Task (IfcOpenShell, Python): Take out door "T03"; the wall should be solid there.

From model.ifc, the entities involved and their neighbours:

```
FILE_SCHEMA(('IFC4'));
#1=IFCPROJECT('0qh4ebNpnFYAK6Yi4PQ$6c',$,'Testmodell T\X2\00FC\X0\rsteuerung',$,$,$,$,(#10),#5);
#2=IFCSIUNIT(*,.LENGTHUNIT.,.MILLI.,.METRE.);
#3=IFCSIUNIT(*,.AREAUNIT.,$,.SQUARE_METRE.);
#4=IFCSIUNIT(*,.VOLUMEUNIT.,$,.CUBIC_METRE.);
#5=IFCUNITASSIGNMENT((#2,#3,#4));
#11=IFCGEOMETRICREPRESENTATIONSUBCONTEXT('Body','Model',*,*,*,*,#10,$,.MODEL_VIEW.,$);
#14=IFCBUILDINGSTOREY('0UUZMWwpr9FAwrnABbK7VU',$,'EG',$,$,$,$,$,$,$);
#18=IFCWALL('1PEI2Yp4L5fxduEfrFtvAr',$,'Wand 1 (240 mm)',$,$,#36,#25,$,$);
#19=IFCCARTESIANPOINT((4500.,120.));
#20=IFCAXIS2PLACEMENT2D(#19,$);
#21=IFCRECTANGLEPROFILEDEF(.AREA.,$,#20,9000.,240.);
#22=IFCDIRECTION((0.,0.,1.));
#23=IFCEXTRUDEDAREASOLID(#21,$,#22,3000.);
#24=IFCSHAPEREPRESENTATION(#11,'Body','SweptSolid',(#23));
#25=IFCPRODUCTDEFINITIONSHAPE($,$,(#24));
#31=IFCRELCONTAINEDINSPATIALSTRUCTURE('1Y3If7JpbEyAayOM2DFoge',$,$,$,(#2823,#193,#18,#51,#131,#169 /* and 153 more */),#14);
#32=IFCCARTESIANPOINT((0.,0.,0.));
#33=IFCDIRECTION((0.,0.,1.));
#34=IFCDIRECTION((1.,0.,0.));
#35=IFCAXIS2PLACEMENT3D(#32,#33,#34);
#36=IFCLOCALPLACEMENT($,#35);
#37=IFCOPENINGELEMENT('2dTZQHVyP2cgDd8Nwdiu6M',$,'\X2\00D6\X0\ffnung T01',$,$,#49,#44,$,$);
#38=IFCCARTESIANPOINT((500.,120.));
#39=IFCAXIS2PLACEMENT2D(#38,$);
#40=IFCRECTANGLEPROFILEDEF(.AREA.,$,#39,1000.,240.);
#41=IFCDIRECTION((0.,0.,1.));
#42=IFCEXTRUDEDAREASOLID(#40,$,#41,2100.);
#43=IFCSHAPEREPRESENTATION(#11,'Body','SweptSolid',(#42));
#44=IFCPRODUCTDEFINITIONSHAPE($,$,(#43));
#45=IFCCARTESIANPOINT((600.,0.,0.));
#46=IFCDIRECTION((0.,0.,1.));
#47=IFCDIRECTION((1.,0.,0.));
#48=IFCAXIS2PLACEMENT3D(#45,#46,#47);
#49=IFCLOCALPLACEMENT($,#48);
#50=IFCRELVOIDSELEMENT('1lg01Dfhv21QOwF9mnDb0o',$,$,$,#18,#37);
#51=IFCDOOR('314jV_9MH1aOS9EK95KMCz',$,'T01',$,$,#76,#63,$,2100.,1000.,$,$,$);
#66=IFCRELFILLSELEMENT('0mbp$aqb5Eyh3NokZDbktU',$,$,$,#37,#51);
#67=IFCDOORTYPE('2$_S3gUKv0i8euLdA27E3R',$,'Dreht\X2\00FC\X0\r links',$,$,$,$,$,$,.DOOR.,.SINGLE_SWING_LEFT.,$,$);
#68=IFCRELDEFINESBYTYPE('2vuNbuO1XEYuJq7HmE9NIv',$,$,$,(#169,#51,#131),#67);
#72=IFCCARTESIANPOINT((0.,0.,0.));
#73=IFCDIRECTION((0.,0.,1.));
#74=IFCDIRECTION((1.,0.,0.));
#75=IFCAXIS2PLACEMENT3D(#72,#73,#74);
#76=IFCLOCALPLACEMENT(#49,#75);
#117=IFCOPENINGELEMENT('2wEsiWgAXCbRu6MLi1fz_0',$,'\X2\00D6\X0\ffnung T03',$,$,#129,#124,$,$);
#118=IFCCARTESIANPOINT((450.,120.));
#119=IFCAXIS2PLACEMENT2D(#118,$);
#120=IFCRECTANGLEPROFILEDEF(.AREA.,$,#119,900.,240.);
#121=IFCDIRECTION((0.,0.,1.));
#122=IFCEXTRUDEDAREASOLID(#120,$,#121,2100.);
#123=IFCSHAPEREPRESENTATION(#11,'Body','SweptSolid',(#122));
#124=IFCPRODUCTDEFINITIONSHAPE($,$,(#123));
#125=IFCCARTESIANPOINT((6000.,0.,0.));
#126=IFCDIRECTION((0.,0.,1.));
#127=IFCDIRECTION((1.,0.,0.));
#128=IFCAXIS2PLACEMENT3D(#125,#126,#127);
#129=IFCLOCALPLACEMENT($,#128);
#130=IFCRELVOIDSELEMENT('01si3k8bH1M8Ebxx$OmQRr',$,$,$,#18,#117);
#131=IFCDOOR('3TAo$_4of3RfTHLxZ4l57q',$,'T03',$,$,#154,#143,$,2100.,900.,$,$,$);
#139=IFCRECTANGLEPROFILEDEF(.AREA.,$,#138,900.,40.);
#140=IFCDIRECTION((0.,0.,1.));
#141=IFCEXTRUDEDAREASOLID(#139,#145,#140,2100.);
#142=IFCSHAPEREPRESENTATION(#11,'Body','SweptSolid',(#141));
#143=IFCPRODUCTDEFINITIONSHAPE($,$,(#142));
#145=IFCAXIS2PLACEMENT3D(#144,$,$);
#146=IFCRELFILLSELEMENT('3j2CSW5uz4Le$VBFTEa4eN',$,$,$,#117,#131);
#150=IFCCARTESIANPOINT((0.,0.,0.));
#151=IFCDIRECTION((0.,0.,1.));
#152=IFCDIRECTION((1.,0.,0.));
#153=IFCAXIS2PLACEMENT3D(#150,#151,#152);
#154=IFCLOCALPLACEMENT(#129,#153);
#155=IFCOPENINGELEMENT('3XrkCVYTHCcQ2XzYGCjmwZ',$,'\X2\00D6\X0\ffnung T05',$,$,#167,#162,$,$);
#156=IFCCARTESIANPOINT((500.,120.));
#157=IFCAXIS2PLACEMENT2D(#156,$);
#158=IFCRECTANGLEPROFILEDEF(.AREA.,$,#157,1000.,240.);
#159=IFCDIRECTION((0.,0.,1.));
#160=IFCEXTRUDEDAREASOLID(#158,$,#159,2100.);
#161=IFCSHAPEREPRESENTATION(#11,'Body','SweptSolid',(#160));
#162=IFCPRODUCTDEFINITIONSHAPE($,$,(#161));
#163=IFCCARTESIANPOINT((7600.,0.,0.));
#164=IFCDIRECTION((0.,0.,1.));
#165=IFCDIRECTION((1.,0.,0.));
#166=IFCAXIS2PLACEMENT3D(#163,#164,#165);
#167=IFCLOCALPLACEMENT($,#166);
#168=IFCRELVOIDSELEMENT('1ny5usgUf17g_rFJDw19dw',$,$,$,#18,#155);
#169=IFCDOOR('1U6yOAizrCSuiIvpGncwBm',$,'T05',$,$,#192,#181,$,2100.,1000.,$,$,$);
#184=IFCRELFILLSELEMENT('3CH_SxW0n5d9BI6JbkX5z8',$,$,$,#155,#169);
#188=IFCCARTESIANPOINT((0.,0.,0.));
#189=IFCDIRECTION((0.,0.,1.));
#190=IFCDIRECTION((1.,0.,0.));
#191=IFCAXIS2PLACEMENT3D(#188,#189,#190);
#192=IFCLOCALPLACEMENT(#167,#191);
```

```python
import ifcopenshell
import ifcopenshell.api.feature
import ifcopenshell.api.root
import ifcopenshell.geom
import ifcopenshell.util.shape

model = ifcopenshell.open("model.ifc")
settings = ifcopenshell.geom.settings()


def volume(element):
    """Net volume in cubic metres, openings subtracted."""
    shape = ifcopenshell.geom.create_shape(settings, element)
    return ifcopenshell.util.shape.get_volume(shape.geometry)


door = model.by_id(131)
opening = door.FillsVoids[0].RelatingOpeningElement
wall = opening.VoidsElements[0].RelatingBuildingElement
before = volume(wall)

ifcopenshell.api.root.remove_product(model, product=door)
ifcopenshell.api.feature.remove_feature(model, feature=opening)

after = volume(wall)

print(f"wall volume {before:.3f} -> {after:.3f} m3")

model.write("model_rev.ifc")
```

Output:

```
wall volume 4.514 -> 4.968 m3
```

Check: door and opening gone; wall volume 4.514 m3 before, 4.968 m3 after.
